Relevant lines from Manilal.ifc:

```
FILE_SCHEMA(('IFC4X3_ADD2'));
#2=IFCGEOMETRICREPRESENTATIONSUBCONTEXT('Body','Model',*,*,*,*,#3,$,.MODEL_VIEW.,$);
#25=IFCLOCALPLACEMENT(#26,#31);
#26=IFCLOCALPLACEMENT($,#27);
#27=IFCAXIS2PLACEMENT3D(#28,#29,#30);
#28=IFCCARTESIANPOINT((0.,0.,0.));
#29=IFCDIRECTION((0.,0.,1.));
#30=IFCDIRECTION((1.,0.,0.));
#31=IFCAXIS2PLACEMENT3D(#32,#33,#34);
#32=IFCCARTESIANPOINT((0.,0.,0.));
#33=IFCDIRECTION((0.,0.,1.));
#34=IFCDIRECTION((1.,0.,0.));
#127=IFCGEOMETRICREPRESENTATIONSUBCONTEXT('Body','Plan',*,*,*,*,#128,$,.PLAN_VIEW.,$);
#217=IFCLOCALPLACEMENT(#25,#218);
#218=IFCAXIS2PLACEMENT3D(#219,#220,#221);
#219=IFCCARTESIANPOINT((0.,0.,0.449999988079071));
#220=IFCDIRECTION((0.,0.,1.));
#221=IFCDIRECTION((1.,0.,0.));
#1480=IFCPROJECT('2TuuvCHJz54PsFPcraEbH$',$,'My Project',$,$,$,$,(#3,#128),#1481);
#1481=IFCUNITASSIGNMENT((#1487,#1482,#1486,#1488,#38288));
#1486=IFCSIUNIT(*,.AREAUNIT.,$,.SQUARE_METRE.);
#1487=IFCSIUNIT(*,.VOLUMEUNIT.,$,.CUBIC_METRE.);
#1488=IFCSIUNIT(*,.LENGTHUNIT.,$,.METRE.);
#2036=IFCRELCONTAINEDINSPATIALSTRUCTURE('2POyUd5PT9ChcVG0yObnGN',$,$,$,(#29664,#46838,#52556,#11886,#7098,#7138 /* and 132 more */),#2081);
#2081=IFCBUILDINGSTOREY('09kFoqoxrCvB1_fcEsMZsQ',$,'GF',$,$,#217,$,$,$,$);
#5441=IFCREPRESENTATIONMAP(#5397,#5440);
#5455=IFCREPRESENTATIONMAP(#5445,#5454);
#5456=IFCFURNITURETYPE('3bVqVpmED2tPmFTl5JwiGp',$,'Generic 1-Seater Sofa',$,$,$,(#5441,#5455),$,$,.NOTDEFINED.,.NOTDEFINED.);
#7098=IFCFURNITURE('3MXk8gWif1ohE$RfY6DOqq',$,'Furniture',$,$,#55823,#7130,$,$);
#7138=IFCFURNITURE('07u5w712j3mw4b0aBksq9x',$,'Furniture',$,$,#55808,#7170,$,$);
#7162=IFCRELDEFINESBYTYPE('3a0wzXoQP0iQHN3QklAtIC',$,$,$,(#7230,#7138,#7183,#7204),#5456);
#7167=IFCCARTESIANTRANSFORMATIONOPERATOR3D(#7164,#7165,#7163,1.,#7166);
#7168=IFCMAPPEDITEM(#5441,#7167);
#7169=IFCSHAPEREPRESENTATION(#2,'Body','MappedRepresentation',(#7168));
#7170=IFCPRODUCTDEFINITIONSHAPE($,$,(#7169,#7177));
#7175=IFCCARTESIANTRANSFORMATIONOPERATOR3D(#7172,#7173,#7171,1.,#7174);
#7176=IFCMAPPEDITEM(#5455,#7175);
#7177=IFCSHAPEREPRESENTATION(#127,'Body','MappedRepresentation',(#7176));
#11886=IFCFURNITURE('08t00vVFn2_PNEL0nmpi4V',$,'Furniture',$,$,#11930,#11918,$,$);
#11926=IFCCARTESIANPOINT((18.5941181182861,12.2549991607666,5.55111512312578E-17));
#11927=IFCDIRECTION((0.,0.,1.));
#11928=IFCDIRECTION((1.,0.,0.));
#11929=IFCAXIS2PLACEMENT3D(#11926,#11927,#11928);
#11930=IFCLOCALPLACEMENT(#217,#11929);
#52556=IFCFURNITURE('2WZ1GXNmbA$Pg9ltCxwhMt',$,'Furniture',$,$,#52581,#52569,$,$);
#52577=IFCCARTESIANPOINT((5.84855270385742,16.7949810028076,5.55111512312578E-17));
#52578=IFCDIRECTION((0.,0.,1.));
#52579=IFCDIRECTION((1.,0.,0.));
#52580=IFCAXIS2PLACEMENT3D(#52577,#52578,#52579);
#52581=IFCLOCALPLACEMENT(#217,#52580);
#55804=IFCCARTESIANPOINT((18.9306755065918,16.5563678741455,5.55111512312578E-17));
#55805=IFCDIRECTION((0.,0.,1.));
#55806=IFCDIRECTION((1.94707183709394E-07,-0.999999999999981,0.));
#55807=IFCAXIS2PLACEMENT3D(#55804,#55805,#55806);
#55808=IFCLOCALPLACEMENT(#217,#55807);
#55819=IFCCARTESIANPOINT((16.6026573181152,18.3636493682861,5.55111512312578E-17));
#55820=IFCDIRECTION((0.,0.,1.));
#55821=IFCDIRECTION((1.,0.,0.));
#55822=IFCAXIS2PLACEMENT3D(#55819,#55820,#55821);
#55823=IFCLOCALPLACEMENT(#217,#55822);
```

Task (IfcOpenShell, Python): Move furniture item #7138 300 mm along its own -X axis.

```python
import ifcopenshell
import ifcopenshell.api.geometry
import ifcopenshell.util.placement
import ifcopenshell.util.unit

model = ifcopenshell.open("Manilal.ifc")
unit_scale = ifcopenshell.util.unit.calculate_unit_scale(model)

item = model.by_guid("07u5w712j3mw4b0aBksq9x")
matrix = ifcopenshell.util.placement.get_local_placement(item.ObjectPlacement)
matrix[:3, 3] -= matrix[:3, 0] * 0.3 / unit_scale
ifcopenshell.api.geometry.edit_object_placement(model, product=item, matrix=matrix, is_si=False)

print(ifcopenshell.util.placement.get_local_placement(item.ObjectPlacement).round(3) + 0.0)

model.write("Manilal_v2.ifc")
```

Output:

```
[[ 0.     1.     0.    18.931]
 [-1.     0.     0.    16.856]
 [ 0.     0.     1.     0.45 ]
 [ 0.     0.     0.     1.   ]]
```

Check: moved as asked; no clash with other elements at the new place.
